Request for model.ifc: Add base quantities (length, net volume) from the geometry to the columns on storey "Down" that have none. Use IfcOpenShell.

First a look at what the model holds.

```python
import ifcopenshell
import ifcopenshell.util.element
import ifcopenshell.util.unit

model = ifcopenshell.open("model.ifc")
print(model.schema)
for unit_type in ("LENGTHUNIT", "AREAUNIT", "VOLUMEUNIT"):
    print(unit_type, ifcopenshell.util.unit.calculate_unit_scale(model, unit_type))
storey = next(s for s in model.by_type("IfcBuildingStorey") if s.Name == "Down")
columns = [e for e in ifcopenshell.util.element.get_decomposition(storey) if e.is_a("IfcColumn")]
for e in sorted(columns, key=lambda e: e.id()):
    print(e.id(), e.is_a(), e.Name, list(ifcopenshell.util.element.get_psets(e, qtos_only=True)), sep=" | ")
```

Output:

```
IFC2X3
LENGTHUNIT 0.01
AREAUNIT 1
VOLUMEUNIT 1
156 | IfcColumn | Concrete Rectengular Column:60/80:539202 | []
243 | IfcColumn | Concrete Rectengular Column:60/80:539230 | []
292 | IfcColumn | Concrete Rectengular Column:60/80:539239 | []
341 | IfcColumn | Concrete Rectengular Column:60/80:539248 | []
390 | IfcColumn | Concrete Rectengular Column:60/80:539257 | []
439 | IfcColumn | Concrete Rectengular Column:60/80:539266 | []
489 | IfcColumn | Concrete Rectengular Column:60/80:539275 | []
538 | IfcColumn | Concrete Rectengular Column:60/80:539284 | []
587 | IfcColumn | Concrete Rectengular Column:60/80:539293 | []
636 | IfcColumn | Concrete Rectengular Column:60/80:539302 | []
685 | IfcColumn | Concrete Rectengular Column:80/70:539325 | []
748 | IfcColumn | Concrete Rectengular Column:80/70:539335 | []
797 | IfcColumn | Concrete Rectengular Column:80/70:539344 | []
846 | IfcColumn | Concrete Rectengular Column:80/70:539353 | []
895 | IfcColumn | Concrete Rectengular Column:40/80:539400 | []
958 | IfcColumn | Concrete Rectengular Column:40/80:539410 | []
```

```python
import ifcopenshell
import ifcopenshell.api.pset
import ifcopenshell.geom
import ifcopenshell.util.element
import ifcopenshell.util.shape
import ifcopenshell.util.unit

model = ifcopenshell.open("model.ifc")
unit_scale = ifcopenshell.util.unit.calculate_unit_scale(model)
volume_scale = ifcopenshell.util.unit.calculate_unit_scale(model, "VOLUMEUNIT")
settings = ifcopenshell.geom.settings()

storey = next(s for s in model.by_type("IfcBuildingStorey") if s.Name == "Down")
columns = [e for e in ifcopenshell.util.element.get_decomposition(storey) if e.is_a("IfcColumn")]

for e in sorted(columns, key=lambda e: e.id()):
    if ifcopenshell.util.element.get_psets(e, qtos_only=True, should_inherit=False):
        continue
    # Geometry comes back in metres, in the element's own axes.
    shape = ifcopenshell.geom.create_shape(settings, e)
    values = {
        "Length": ifcopenshell.util.shape.get_z(shape.geometry) / unit_scale,
        "NetVolume": ifcopenshell.util.shape.get_volume(shape.geometry) / volume_scale,
    }
    qto = ifcopenshell.api.pset.add_qto(model, product=e, name="BaseQuantities")
    ifcopenshell.api.pset.edit_qto(model, qto=qto, properties=values)
    print(e.id(), {k: round(v, 3) for k, v in values.items()})

model.write("model_v2.ifc")
```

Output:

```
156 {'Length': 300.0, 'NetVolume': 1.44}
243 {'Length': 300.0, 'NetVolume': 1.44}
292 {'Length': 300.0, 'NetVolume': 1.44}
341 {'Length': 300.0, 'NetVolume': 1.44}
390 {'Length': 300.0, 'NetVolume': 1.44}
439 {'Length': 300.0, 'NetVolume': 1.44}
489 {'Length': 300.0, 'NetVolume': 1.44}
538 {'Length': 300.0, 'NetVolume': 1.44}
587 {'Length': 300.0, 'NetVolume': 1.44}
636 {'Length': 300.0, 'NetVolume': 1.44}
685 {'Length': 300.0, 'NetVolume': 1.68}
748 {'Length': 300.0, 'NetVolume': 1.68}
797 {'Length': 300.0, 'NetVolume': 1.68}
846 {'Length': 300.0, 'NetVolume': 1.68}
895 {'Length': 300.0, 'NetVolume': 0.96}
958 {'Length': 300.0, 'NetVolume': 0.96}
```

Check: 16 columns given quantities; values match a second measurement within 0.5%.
